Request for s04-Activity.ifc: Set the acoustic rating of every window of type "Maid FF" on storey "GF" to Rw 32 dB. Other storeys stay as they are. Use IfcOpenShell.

First a look at what the model holds.

```python
import ifcopenshell
import ifcopenshell.util.element

model = ifcopenshell.open("s04-Activity.ifc")
print(model.schema)
storey = next(s for s in model.by_type("IfcBuildingStorey") if s.Name == "GF")
windows = [e for e in ifcopenshell.util.element.get_decomposition(storey) if e.is_a("IfcWindow")]
seen = {}
for e in windows:
    element_type = ifcopenshell.util.element.get_type(e)
    key = (element_type.Name if element_type != e and element_type else None, ifcopenshell.util.element.get_pset(e, "Pset_WindowCommon", "AcousticRating"))
    seen[key] = seen.get(key, 0) + 1
for (name, value), count in sorted(seen.items(), key=str):
    print(count, "x", name, "|", value)
```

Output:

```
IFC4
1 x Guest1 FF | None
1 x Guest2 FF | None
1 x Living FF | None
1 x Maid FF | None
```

```python
import ifcopenshell
import ifcopenshell.api.pset
import ifcopenshell.util.element

model = ifcopenshell.open("s04-Activity.ifc")

storey = next(s for s in model.by_type("IfcBuildingStorey") if s.Name == "GF")
windows = [e for e in ifcopenshell.util.element.get_decomposition(storey) if e.is_a("IfcWindow")]

count = 0
for e in windows:
    element_type = ifcopenshell.util.element.get_type(e)
    if element_type in (None, e) or element_type.Name != "Maid FF":
        continue
    # add_pset returns the element's existing set when there is one.
    pset = ifcopenshell.api.pset.add_pset(model, product=e, name="Pset_WindowCommon")
    ifcopenshell.api.pset.edit_pset(model, pset=pset, properties={"AcousticRating": "Rw 32 dB"})
    count += 1

print(count, "windows updated")

model.write("s04-Activity_v2.ifc")
```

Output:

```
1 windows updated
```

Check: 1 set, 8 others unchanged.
